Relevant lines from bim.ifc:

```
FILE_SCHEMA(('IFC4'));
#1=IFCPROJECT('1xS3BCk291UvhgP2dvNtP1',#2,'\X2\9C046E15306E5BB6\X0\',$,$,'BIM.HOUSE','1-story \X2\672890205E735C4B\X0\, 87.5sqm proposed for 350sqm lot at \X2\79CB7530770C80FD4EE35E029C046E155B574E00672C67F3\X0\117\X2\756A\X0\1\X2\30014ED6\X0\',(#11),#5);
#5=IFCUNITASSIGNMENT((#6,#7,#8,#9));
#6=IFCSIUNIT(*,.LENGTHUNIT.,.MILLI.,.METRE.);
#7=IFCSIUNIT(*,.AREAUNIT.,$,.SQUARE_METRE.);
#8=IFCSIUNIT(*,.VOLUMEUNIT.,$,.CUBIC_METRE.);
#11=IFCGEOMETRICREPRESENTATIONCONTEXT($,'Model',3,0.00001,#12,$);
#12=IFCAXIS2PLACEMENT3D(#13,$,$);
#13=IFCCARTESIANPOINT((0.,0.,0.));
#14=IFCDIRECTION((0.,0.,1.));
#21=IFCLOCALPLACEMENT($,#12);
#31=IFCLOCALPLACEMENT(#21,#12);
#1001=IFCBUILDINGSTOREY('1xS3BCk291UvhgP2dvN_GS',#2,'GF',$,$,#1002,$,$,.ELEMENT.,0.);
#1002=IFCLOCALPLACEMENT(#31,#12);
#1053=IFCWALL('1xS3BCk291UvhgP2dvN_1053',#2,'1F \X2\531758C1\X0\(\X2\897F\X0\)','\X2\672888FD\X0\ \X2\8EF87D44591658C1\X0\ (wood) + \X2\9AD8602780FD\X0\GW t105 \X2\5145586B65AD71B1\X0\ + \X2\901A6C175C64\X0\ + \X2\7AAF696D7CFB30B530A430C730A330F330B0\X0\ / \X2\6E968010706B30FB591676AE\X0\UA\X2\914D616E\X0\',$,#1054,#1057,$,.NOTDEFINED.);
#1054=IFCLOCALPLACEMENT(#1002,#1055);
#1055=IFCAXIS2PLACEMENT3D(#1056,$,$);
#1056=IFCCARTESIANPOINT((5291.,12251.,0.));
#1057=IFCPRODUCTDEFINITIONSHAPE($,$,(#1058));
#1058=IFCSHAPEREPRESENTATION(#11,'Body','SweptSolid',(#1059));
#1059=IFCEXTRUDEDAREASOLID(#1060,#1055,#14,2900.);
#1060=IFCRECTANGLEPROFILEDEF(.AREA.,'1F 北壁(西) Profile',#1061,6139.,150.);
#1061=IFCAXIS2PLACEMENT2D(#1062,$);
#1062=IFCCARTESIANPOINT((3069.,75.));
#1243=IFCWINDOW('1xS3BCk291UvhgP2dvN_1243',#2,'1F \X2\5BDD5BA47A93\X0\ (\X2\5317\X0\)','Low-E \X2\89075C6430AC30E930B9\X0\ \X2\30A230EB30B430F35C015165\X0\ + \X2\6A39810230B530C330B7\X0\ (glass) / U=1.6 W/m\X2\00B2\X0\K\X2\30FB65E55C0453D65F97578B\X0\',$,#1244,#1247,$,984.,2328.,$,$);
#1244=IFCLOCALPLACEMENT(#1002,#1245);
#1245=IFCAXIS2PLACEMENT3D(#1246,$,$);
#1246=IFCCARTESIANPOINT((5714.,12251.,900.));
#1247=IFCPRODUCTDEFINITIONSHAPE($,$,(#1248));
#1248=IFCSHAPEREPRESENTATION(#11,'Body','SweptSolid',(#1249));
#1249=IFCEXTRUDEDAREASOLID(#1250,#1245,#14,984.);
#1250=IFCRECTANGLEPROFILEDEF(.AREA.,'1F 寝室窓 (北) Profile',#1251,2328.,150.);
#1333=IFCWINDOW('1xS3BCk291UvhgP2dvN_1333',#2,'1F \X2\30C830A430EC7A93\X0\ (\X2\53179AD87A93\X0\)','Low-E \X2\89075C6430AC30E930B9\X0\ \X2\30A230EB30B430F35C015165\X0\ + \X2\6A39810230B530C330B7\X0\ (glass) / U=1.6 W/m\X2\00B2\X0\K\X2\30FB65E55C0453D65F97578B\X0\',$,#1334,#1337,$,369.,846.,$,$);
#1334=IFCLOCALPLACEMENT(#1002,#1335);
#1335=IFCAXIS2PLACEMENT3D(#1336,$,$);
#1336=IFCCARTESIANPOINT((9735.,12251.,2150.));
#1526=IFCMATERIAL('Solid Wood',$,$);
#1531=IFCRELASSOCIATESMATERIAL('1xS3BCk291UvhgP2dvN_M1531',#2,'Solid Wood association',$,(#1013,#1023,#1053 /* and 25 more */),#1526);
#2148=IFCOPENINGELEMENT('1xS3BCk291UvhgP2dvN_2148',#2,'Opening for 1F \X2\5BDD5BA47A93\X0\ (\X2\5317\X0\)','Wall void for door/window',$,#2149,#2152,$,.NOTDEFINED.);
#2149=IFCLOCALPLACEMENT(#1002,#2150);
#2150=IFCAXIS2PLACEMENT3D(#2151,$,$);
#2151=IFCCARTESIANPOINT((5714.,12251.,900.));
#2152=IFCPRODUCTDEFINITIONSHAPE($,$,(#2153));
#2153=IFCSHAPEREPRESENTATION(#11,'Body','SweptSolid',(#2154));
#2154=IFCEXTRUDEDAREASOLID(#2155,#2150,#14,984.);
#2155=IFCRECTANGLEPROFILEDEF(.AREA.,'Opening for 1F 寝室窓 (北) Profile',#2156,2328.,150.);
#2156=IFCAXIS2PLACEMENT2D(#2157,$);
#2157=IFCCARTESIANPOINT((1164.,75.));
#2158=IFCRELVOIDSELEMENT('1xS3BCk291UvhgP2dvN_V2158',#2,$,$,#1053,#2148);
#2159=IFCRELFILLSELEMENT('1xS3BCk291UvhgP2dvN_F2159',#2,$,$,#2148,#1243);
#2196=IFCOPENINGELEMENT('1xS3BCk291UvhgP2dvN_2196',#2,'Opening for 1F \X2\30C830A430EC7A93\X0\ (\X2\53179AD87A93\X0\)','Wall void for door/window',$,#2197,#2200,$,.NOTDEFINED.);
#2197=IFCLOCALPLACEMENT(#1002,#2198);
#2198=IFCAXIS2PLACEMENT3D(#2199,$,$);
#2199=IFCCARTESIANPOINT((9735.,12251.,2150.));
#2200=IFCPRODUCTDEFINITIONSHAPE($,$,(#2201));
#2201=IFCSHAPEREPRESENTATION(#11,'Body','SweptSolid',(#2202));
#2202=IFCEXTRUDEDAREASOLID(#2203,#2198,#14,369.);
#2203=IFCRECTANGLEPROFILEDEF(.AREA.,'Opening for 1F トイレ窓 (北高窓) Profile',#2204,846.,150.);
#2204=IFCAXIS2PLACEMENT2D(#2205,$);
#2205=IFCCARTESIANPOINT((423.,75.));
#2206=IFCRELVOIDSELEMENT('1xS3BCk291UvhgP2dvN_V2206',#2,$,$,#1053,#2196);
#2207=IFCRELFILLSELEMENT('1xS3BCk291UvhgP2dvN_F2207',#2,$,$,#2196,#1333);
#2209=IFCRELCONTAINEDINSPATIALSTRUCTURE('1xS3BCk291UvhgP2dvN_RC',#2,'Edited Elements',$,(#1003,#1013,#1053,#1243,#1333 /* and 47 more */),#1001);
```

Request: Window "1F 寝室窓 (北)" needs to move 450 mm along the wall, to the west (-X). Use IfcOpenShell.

```python
import ifcopenshell
import ifcopenshell.api.geometry
import ifcopenshell.util.placement

model = ifcopenshell.open("bim.ifc")

window = model.by_guid("1xS3BCk291UvhgP2dvN_1243")
opening = window.FillsVoids[0].RelatingOpeningElement
wall = opening.VoidsElements[0].RelatingBuildingElement

wall_matrix = ifcopenshell.util.placement.get_local_placement(wall.ObjectPlacement)
shift = wall_matrix[:3, 0] * -450.0
before = ifcopenshell.util.placement.get_local_placement(window.ObjectPlacement)[:3, 3].copy()

# The window is not placed relative to its opening, so move both.
for product in (opening, window):
    matrix = ifcopenshell.util.placement.get_local_placement(product.ObjectPlacement)
    matrix[:3, 3] += shift
    ifcopenshell.api.geometry.edit_object_placement(model, product=product, matrix=matrix, is_si=False)

after = ifcopenshell.util.placement.get_local_placement(window.ObjectPlacement)[:3, 3]
print("window moved by", (after - before).round(3) + 0.0)

model.write("bim_v2.ifc")
```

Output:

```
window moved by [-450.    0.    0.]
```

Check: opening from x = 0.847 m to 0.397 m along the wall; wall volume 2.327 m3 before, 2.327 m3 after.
